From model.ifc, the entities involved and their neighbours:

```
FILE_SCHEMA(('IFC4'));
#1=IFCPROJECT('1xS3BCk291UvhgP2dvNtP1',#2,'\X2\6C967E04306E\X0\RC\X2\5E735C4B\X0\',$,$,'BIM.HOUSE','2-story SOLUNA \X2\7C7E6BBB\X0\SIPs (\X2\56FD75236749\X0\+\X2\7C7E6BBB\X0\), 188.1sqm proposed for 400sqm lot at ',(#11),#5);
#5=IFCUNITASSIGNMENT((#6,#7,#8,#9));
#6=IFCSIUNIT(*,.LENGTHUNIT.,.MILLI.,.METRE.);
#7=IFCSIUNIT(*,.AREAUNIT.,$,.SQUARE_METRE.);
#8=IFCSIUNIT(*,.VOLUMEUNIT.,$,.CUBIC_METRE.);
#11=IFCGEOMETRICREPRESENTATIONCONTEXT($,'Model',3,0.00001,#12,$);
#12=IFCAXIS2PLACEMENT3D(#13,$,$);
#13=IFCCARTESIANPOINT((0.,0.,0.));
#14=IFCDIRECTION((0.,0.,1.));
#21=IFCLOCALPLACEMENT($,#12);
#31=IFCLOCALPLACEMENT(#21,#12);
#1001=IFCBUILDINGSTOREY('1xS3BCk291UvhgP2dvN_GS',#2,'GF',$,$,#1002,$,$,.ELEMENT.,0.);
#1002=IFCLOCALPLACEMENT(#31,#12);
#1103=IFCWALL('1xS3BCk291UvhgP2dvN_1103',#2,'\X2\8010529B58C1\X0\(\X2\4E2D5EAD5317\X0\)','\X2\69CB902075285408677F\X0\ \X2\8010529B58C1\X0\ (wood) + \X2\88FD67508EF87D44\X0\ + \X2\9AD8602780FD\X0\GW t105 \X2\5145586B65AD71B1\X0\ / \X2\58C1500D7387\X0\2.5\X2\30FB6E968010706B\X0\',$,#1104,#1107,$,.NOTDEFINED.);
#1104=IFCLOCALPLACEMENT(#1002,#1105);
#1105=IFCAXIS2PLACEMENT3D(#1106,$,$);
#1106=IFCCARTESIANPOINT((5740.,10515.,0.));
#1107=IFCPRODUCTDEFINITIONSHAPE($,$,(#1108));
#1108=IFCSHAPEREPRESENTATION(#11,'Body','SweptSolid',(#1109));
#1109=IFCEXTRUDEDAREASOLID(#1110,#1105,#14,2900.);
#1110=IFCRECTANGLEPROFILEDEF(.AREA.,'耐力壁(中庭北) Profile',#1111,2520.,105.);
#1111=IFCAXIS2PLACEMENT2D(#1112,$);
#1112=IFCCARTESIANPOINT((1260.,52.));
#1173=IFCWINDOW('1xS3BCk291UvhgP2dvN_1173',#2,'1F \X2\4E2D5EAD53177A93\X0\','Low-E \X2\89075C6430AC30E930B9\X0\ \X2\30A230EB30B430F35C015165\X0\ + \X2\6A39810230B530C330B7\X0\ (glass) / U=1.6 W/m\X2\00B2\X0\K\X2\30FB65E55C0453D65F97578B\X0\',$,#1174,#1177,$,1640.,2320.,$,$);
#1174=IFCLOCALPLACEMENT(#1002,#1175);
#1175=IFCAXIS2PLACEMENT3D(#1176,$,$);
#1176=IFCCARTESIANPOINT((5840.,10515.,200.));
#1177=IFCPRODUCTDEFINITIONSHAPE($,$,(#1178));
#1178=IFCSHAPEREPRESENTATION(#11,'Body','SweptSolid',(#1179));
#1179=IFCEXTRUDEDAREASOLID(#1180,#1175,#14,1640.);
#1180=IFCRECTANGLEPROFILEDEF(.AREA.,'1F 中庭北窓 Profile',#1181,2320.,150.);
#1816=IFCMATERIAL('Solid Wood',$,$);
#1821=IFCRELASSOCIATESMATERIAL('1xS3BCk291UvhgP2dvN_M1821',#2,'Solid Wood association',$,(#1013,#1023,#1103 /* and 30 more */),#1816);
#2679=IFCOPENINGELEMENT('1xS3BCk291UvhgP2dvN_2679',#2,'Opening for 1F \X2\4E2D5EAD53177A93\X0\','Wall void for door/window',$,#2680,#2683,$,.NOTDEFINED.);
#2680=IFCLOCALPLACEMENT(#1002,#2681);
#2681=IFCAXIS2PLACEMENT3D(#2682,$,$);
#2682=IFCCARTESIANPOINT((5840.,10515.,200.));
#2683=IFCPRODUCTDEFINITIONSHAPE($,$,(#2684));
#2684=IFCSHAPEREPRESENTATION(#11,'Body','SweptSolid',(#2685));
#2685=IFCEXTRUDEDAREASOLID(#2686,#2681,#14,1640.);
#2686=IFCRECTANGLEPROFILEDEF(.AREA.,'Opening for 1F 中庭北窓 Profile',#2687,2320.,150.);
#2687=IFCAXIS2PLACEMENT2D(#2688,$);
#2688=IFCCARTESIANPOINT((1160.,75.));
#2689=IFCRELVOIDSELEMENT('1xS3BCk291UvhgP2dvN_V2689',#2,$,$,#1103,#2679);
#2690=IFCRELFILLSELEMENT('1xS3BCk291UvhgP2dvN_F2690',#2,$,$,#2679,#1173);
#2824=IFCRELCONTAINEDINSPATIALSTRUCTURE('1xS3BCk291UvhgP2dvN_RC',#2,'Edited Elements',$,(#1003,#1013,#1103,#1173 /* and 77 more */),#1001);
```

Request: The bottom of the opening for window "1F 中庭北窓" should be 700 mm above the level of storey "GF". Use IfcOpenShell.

```python
import numpy as np
import ifcopenshell
import ifcopenshell.api.geometry
import ifcopenshell.geom
import ifcopenshell.util.element
import ifcopenshell.util.placement
import ifcopenshell.util.shape
import ifcopenshell.util.unit

model = ifcopenshell.open("model.ifc")
unit_scale = ifcopenshell.util.unit.calculate_unit_scale(model)

window = model.by_id(1173)
opening = window.FillsVoids[0].RelatingOpeningElement
storey = ifcopenshell.util.element.get_container(window, ifc_class="IfcBuildingStorey")
level = ifcopenshell.util.placement.get_local_placement(storey.ObjectPlacement)[2, 3]

# The opening's origin need not be at the sill, so measure its lowest point.
shape = ifcopenshell.geom.create_shape(ifcopenshell.geom.settings(), opening)
bottom = ifcopenshell.util.shape.get_shape_bottom_elevation(shape, shape.geometry) / unit_scale
dz = level + 700.0 - bottom

shift = np.array([0.0, 0.0, dz])
# The window is not placed relative to its opening, so move both.
for product in (opening, window):
    matrix = ifcopenshell.util.placement.get_local_placement(product.ObjectPlacement)
    matrix[:3, 3] += shift
    ifcopenshell.api.geometry.edit_object_placement(model, product=product, matrix=matrix, is_si=False)

print(f"moved by {dz * unit_scale:+.3f} m")

model.write("model_updated.ifc")
```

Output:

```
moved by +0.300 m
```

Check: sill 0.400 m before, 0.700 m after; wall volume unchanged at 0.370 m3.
